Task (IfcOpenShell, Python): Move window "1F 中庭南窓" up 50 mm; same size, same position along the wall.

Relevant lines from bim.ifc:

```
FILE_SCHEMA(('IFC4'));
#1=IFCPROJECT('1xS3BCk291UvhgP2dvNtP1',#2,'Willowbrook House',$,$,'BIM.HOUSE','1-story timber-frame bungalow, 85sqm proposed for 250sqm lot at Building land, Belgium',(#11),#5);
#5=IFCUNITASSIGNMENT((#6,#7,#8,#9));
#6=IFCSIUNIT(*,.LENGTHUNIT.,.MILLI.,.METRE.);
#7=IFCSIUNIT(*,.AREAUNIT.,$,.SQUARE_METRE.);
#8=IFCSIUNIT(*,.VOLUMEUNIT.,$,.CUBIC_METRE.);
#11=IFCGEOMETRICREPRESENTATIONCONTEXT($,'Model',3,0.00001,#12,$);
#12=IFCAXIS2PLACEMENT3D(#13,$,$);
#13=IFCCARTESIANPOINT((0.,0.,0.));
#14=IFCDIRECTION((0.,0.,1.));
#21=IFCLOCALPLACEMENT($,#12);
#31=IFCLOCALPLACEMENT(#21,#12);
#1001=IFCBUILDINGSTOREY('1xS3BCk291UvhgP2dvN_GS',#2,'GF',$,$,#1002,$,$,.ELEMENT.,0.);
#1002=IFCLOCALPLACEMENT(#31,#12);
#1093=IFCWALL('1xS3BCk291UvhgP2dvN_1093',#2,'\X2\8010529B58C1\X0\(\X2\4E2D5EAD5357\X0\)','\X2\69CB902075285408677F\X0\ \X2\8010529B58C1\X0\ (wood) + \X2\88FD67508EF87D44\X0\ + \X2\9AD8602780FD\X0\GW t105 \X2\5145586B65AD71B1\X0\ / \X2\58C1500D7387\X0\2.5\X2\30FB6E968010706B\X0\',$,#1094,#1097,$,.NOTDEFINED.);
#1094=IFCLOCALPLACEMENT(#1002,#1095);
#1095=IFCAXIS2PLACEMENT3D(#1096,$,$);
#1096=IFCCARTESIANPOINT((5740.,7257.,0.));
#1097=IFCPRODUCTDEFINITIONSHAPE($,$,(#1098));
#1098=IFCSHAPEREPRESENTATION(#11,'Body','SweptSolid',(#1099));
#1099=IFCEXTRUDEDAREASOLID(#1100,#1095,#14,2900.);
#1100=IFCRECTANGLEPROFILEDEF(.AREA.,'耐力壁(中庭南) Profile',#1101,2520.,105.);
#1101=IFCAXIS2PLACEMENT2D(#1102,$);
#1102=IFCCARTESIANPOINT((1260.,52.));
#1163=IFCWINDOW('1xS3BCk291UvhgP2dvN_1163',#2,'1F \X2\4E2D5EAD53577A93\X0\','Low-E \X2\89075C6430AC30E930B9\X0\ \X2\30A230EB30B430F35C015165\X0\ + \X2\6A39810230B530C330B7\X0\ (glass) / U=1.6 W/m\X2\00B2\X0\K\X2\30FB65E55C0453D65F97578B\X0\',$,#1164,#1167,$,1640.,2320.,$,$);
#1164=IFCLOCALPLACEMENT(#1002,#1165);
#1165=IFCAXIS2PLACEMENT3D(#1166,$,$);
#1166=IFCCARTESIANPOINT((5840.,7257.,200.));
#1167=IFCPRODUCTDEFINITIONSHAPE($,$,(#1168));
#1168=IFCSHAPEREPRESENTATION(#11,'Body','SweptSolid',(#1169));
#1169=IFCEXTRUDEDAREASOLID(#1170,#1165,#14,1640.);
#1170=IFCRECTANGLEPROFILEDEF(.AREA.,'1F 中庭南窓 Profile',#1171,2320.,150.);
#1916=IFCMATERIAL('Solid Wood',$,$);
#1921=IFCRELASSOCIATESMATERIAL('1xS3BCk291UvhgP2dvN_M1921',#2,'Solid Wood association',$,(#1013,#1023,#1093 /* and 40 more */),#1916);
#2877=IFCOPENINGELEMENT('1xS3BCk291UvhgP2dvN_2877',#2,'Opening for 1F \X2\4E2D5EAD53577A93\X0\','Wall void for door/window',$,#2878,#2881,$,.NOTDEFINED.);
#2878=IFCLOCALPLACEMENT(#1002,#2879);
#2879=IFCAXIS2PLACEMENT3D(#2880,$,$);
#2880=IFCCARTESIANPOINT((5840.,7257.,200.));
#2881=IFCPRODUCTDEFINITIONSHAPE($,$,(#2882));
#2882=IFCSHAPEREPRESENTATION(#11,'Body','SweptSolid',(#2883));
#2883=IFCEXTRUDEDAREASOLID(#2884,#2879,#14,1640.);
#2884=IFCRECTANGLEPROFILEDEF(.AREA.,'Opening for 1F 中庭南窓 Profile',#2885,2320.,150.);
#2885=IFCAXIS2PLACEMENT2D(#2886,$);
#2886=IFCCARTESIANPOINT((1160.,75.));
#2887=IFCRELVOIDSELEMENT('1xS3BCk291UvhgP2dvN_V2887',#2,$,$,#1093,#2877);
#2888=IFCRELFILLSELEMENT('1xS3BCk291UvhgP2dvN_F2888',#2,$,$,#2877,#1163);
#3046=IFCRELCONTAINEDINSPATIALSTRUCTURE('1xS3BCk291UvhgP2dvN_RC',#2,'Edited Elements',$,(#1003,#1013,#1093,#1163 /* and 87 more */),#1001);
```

```python
import numpy as np
import ifcopenshell
import ifcopenshell.api.geometry
import ifcopenshell.util.placement
import ifcopenshell.util.unit

model = ifcopenshell.open("bim.ifc")
unit_scale = ifcopenshell.util.unit.calculate_unit_scale(model)

window = model.by_id(1163)
opening = window.FillsVoids[0].RelatingOpeningElement
dz = 0.05 / unit_scale

shift = np.array([0.0, 0.0, dz])
# The window is not placed relative to its opening, so move both.
for product in (opening, window):
    matrix = ifcopenshell.util.placement.get_local_placement(product.ObjectPlacement)
    matrix[:3, 3] += shift
    ifcopenshell.api.geometry.edit_object_placement(model, product=product, matrix=matrix, is_si=False)

print(f"moved by {dz * unit_scale:+.3f} m")

model.write("bim_v2.ifc")
```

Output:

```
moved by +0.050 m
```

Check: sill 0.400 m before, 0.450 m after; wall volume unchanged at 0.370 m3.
